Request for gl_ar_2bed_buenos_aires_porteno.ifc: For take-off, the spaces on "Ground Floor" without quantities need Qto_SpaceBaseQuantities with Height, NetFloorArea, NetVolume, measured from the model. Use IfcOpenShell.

First a look at what the model holds.

```python
import ifcopenshell
import ifcopenshell.util.element
import ifcopenshell.util.unit

model = ifcopenshell.open("gl_ar_2bed_buenos_aires_porteno.ifc")
print(model.schema)
for unit_type in ("LENGTHUNIT", "AREAUNIT", "VOLUMEUNIT"):
    print(unit_type, ifcopenshell.util.unit.calculate_unit_scale(model, unit_type))
storey = next(s for s in model.by_type("IfcBuildingStorey") if s.Name == "Ground Floor")
spaces = [e for e in ifcopenshell.util.element.get_decomposition(storey) if e.is_a("IfcSpace")]
for e in sorted(spaces, key=lambda e: e.id()):
    print(e.id(), e.is_a(), e.Name, list(ifcopenshell.util.element.get_psets(e, qtos_only=True)), sep=" | ")
```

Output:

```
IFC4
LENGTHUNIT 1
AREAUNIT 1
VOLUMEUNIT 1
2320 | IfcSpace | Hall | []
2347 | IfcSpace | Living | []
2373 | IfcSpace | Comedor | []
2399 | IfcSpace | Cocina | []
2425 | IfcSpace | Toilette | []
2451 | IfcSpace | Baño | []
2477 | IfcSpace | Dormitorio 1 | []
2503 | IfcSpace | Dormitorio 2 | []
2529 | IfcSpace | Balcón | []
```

```python
import ifcopenshell
import ifcopenshell.api.pset
import ifcopenshell.geom
import ifcopenshell.util.element
import ifcopenshell.util.shape
import ifcopenshell.util.unit

model = ifcopenshell.open("gl_ar_2bed_buenos_aires_porteno.ifc")
unit_scale = ifcopenshell.util.unit.calculate_unit_scale(model)
area_scale = ifcopenshell.util.unit.calculate_unit_scale(model, "AREAUNIT")
volume_scale = ifcopenshell.util.unit.calculate_unit_scale(model, "VOLUMEUNIT")
settings = ifcopenshell.geom.settings()

storey = next(s for s in model.by_type("IfcBuildingStorey") if s.Name == "Ground Floor")
spaces = [e for e in ifcopenshell.util.element.get_decomposition(storey) if e.is_a("IfcSpace")]

for e in sorted(spaces, key=lambda e: e.id()):
    if ifcopenshell.util.element.get_psets(e, qtos_only=True, should_inherit=False):
        continue
    # Geometry comes back in metres, in the element's own axes.
    shape = ifcopenshell.geom.create_shape(settings, e)
    values = {
        "Height": ifcopenshell.util.shape.get_z(shape.geometry) / unit_scale,
        "NetFloorArea": ifcopenshell.util.shape.get_footprint_area(shape.geometry) / area_scale,
        "NetVolume": ifcopenshell.util.shape.get_volume(shape.geometry) / volume_scale,
    }
    qto = ifcopenshell.api.pset.add_qto(model, product=e, name="Qto_SpaceBaseQuantities")
    ifcopenshell.api.pset.edit_qto(model, qto=qto, properties=values)
    print(e.id(), {k: round(v, 3) for k, v in values.items()})

model.write("gl_ar_2bed_buenos_aires_porteno-out.ifc")
```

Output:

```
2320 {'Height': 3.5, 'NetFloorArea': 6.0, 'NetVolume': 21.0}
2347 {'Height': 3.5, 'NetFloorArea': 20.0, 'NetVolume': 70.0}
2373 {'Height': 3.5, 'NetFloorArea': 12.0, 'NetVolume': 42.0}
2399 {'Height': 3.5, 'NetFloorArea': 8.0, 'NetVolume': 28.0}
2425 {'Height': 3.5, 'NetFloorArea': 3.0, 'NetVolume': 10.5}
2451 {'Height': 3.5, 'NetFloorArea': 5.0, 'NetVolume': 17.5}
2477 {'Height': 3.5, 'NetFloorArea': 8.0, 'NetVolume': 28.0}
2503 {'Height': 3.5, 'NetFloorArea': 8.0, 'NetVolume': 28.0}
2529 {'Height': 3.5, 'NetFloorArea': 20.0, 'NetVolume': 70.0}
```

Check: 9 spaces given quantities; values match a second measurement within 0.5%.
